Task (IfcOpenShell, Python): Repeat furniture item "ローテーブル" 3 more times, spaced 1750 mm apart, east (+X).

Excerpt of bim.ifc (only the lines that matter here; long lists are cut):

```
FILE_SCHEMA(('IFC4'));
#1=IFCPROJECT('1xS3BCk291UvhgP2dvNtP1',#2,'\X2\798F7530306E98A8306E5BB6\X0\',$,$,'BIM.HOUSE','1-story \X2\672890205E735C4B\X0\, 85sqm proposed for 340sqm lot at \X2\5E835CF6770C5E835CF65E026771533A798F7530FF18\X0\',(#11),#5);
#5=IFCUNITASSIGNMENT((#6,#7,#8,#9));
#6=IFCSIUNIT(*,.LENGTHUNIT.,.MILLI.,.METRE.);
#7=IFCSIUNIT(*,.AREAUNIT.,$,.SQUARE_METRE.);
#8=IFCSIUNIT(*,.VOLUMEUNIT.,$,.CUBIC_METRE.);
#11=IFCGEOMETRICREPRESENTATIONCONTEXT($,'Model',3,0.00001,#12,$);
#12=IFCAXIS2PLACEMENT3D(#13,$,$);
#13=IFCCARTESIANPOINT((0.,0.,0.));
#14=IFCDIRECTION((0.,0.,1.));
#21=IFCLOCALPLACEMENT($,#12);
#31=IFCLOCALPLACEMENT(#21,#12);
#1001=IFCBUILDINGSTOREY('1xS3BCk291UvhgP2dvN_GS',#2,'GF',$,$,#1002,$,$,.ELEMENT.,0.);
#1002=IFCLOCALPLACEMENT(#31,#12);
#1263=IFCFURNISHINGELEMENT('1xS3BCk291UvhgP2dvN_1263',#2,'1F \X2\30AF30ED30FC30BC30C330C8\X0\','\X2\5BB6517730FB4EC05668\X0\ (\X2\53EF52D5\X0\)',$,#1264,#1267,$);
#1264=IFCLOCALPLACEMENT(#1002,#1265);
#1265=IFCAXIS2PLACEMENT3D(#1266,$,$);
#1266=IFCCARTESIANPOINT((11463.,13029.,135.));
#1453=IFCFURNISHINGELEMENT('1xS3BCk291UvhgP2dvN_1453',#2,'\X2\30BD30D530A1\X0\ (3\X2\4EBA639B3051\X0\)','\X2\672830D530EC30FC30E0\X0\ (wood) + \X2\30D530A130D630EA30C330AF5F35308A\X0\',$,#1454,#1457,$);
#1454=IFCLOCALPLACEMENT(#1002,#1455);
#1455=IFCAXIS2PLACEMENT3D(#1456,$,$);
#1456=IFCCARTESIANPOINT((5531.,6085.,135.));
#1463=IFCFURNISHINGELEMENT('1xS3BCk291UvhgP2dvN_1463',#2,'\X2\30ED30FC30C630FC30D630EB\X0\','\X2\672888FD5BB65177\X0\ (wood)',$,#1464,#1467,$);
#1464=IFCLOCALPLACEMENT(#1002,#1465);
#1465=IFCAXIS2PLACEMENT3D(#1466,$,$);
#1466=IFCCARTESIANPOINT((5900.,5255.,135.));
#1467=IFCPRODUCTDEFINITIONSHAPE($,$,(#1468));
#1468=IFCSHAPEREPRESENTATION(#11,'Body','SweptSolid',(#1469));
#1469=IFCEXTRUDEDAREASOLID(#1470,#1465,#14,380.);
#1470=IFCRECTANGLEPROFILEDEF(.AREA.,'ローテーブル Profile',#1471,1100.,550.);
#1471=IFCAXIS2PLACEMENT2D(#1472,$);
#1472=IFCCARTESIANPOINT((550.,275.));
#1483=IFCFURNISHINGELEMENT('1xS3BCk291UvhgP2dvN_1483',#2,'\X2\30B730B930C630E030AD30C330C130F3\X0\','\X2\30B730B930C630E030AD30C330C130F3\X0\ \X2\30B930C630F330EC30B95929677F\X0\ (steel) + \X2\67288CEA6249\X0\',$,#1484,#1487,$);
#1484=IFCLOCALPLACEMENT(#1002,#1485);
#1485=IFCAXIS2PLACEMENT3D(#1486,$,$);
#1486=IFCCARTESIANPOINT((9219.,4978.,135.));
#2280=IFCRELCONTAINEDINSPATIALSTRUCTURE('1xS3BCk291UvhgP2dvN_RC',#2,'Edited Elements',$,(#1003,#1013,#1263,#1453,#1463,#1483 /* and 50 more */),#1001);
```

```python
import numpy as np
import ifcopenshell
import ifcopenshell.api.geometry
import ifcopenshell.api.root
import ifcopenshell.util.element
import ifcopenshell.util.placement
import ifcopenshell.util.unit

model = ifcopenshell.open("bim.ifc")
unit_scale = ifcopenshell.util.unit.calculate_unit_scale(model)


def reuse_history(source, copy):
    """copy_class also copies each property set's owner history, people and application; keep the originals."""
    for rel in copy.IsDefinedBy:
        if rel.is_a("IfcRelDefinesByProperties") and (history := rel.RelatingPropertyDefinition.OwnerHistory):
            rel.RelatingPropertyDefinition.OwnerHistory = source.OwnerHistory
            ifcopenshell.util.element.remove_deep2(model, history)


source = model.by_id(1463)
base = ifcopenshell.util.placement.get_local_placement(source.ObjectPlacement)
step = np.array([1.0, 0.0, 0.0]) * 1.75 / unit_scale

for i in range(1, 4):
    copy = ifcopenshell.api.root.copy_class(model, product=source)
    copy.Representation = ifcopenshell.util.element.copy_deep(
        model, source.Representation, exclude=["IfcGeometricRepresentationContext", "IfcRepresentationMap"]
    )
    reuse_history(source, copy)
    matrix = base.copy()
    matrix[:3, 3] += i * step
    print("added at", matrix[:3, 3].round(3) + 0.0)
    ifcopenshell.api.geometry.edit_object_placement(model, product=copy, matrix=matrix, is_si=False)

model.write("bim-out.ifc")
```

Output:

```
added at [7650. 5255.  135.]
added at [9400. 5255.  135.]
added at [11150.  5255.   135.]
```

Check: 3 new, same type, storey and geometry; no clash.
